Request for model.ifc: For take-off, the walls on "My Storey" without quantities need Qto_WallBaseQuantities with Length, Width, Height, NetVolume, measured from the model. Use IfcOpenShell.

First a look at what the model holds.

```python
import ifcopenshell
import ifcopenshell.util.element
import ifcopenshell.util.unit

model = ifcopenshell.open("model.ifc")
print(model.schema)
for unit_type in ("LENGTHUNIT", "AREAUNIT", "VOLUMEUNIT"):
    print(unit_type, ifcopenshell.util.unit.calculate_unit_scale(model, unit_type))
storey = next(s for s in model.by_type("IfcBuildingStorey") if s.Name == "My Storey")
walls = [e for e in ifcopenshell.util.element.get_decomposition(storey) if e.is_a("IfcWall")]
for e in sorted(walls, key=lambda e: e.id()):
    print(e.id(), e.is_a(), e.Name, list(ifcopenshell.util.element.get_psets(e, qtos_only=True)), sep=" | ")
```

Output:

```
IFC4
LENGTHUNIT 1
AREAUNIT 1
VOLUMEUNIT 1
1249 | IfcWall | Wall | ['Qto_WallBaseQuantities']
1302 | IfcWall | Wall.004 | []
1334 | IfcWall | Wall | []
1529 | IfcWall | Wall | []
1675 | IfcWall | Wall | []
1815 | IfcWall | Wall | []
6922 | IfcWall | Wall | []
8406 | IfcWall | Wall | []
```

```python
import ifcopenshell
import ifcopenshell.api.pset
import ifcopenshell.geom
import ifcopenshell.util.element
import ifcopenshell.util.shape
import ifcopenshell.util.unit

model = ifcopenshell.open("model.ifc")
unit_scale = ifcopenshell.util.unit.calculate_unit_scale(model)
volume_scale = ifcopenshell.util.unit.calculate_unit_scale(model, "VOLUMEUNIT")
settings = ifcopenshell.geom.settings()

storey = next(s for s in model.by_type("IfcBuildingStorey") if s.Name == "My Storey")
walls = [e for e in ifcopenshell.util.element.get_decomposition(storey) if e.is_a("IfcWall")]

for e in sorted(walls, key=lambda e: e.id()):
    if ifcopenshell.util.element.get_psets(e, qtos_only=True, should_inherit=False):
        continue
    # Geometry comes back in metres, in the element's own axes.
    shape = ifcopenshell.geom.create_shape(settings, e)
    values = {
        "Length": ifcopenshell.util.shape.get_x(shape.geometry) / unit_scale,
        "Width": ifcopenshell.util.shape.get_y(shape.geometry) / unit_scale,
        "Height": ifcopenshell.util.shape.get_z(shape.geometry) / unit_scale,
        "NetVolume": ifcopenshell.util.shape.get_volume(shape.geometry) / volume_scale,
    }
    qto = ifcopenshell.api.pset.add_qto(model, product=e, name="Qto_WallBaseQuantities")
    ifcopenshell.api.pset.edit_qto(model, qto=qto, properties=values)
    print(e.id(), {k: round(v, 3) for k, v in values.items()})

model.write("model-out.ifc")
```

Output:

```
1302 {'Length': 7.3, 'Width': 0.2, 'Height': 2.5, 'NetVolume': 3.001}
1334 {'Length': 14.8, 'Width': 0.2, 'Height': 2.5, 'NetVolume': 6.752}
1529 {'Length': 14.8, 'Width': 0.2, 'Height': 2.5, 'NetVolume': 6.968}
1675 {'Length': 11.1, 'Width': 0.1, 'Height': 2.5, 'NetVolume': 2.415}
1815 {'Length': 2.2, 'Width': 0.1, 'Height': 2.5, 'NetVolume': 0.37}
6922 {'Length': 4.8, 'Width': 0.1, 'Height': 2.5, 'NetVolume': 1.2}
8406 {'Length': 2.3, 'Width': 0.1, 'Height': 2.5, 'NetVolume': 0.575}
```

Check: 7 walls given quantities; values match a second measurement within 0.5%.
